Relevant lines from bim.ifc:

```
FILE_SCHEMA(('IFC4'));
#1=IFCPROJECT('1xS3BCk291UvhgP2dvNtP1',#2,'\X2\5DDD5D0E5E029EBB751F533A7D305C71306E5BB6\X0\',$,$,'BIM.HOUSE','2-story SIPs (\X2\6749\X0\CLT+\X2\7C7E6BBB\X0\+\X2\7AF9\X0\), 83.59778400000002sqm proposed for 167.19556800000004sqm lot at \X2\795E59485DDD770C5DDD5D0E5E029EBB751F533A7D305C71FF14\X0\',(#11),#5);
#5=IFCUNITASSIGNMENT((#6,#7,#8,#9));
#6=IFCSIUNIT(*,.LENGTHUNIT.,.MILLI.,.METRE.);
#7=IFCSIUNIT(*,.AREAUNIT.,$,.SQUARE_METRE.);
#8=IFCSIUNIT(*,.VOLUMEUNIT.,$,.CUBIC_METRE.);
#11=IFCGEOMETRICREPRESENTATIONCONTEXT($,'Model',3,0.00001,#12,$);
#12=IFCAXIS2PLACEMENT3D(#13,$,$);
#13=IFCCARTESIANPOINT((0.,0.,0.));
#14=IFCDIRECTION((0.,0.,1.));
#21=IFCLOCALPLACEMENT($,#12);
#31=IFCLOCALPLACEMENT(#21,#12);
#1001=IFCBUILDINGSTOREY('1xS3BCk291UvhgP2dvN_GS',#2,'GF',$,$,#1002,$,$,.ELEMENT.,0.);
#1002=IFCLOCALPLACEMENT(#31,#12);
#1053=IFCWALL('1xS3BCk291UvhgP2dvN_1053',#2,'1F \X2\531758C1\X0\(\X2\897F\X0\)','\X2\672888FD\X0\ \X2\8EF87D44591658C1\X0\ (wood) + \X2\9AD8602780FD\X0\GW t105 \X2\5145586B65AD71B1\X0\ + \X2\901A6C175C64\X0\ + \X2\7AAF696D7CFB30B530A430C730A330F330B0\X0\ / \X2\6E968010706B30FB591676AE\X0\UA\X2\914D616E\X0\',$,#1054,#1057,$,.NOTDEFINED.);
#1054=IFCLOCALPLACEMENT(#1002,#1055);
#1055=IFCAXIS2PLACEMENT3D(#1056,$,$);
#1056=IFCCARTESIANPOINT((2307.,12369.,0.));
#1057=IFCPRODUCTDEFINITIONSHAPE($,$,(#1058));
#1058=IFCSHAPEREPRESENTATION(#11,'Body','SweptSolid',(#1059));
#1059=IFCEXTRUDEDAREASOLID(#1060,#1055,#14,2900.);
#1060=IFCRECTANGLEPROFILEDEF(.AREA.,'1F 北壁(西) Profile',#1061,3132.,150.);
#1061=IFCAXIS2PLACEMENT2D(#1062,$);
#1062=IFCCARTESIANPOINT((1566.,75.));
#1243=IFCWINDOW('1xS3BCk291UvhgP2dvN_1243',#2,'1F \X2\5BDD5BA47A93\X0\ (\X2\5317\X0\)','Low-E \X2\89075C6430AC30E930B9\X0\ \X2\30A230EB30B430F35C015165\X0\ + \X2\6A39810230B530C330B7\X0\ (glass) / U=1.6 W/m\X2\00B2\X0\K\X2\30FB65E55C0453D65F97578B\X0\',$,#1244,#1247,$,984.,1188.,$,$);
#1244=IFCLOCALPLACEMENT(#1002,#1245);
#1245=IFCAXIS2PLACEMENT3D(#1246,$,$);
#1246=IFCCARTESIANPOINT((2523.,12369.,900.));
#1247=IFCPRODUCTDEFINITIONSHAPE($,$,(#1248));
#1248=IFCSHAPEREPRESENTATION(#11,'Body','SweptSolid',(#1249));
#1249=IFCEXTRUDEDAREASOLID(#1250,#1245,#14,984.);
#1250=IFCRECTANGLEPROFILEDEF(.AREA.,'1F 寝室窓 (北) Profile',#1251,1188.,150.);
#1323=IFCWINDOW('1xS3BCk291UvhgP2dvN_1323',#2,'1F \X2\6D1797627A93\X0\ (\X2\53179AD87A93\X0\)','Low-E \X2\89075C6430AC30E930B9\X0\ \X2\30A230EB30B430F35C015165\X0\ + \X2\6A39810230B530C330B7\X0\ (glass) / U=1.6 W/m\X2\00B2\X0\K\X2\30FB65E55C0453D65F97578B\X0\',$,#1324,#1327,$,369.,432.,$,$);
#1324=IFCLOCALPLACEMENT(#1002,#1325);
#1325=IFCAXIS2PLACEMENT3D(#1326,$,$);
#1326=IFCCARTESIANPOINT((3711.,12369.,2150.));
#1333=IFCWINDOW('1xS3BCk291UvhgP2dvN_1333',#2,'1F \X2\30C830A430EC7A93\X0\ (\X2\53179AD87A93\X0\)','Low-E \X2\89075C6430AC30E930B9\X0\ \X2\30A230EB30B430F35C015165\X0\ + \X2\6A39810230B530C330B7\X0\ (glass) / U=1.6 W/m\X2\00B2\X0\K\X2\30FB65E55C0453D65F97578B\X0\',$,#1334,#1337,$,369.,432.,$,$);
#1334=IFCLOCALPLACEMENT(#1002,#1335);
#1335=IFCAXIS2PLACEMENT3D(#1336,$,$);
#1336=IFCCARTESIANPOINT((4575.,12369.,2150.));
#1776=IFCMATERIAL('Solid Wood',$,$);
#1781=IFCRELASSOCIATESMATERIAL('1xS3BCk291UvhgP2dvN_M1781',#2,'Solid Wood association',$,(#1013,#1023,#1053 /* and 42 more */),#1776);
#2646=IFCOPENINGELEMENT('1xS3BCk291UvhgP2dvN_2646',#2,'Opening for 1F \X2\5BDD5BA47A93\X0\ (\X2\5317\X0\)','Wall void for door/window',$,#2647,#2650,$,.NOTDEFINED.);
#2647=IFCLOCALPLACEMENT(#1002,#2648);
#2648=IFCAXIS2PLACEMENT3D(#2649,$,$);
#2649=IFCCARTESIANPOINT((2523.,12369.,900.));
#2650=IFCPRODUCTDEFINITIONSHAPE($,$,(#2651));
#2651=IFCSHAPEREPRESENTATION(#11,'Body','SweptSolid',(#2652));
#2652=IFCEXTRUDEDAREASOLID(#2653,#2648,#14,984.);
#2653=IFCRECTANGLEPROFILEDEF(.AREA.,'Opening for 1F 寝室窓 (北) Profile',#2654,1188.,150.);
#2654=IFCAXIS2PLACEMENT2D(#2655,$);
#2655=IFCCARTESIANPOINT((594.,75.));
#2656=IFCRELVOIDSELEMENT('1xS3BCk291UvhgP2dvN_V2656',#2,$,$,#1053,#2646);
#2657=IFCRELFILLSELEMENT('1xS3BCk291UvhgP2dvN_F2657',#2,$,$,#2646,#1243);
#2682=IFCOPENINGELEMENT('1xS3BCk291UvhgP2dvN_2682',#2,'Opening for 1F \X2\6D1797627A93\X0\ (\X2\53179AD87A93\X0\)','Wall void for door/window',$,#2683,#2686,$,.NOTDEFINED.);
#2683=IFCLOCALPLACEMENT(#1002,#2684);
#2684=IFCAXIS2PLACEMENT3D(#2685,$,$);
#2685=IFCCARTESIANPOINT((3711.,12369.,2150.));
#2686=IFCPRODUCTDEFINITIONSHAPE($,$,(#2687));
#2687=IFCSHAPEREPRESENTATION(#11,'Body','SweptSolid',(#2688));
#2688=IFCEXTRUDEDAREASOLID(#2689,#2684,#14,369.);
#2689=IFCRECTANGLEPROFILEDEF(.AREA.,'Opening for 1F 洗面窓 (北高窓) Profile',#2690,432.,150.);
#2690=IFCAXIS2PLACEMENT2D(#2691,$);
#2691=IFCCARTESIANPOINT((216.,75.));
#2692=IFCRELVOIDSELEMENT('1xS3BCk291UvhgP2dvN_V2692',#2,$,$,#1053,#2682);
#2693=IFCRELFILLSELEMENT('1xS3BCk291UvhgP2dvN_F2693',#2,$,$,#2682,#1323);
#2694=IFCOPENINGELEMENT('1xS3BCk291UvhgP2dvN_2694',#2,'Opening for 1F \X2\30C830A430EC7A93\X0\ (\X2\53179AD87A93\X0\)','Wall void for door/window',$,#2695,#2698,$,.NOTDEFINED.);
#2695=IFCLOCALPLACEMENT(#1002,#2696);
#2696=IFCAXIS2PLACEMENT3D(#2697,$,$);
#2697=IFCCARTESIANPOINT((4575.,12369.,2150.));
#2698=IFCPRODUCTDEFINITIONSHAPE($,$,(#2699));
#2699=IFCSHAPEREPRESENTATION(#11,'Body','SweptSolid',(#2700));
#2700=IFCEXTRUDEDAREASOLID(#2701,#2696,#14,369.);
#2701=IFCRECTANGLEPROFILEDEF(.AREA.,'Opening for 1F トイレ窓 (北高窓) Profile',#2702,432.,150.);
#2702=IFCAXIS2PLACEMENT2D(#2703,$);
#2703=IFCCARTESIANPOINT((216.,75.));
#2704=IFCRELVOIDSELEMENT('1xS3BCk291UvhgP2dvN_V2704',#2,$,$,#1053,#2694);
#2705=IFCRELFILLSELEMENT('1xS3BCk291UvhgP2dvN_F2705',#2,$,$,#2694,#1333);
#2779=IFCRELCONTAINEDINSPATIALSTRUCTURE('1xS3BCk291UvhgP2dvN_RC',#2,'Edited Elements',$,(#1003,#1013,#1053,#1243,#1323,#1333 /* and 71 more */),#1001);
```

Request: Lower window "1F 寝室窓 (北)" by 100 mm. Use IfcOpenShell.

```python
import numpy as np
import ifcopenshell
import ifcopenshell.api.geometry
import ifcopenshell.util.placement
import ifcopenshell.util.unit

model = ifcopenshell.open("bim.ifc")
unit_scale = ifcopenshell.util.unit.calculate_unit_scale(model)

window = model.by_id(1243)
opening = window.FillsVoids[0].RelatingOpeningElement
dz = -0.1 / unit_scale

shift = np.array([0.0, 0.0, dz])
# The window is not placed relative to its opening, so move both.
for product in (opening, window):
    matrix = ifcopenshell.util.placement.get_local_placement(product.ObjectPlacement)
    matrix[:3, 3] += shift
    ifcopenshell.api.geometry.edit_object_placement(model, product=product, matrix=matrix, is_si=False)

print(f"moved by {dz * unit_scale:+.3f} m")

model.write("bim_rev.ifc")
```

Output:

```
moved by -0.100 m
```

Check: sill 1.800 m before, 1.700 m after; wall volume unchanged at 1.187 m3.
